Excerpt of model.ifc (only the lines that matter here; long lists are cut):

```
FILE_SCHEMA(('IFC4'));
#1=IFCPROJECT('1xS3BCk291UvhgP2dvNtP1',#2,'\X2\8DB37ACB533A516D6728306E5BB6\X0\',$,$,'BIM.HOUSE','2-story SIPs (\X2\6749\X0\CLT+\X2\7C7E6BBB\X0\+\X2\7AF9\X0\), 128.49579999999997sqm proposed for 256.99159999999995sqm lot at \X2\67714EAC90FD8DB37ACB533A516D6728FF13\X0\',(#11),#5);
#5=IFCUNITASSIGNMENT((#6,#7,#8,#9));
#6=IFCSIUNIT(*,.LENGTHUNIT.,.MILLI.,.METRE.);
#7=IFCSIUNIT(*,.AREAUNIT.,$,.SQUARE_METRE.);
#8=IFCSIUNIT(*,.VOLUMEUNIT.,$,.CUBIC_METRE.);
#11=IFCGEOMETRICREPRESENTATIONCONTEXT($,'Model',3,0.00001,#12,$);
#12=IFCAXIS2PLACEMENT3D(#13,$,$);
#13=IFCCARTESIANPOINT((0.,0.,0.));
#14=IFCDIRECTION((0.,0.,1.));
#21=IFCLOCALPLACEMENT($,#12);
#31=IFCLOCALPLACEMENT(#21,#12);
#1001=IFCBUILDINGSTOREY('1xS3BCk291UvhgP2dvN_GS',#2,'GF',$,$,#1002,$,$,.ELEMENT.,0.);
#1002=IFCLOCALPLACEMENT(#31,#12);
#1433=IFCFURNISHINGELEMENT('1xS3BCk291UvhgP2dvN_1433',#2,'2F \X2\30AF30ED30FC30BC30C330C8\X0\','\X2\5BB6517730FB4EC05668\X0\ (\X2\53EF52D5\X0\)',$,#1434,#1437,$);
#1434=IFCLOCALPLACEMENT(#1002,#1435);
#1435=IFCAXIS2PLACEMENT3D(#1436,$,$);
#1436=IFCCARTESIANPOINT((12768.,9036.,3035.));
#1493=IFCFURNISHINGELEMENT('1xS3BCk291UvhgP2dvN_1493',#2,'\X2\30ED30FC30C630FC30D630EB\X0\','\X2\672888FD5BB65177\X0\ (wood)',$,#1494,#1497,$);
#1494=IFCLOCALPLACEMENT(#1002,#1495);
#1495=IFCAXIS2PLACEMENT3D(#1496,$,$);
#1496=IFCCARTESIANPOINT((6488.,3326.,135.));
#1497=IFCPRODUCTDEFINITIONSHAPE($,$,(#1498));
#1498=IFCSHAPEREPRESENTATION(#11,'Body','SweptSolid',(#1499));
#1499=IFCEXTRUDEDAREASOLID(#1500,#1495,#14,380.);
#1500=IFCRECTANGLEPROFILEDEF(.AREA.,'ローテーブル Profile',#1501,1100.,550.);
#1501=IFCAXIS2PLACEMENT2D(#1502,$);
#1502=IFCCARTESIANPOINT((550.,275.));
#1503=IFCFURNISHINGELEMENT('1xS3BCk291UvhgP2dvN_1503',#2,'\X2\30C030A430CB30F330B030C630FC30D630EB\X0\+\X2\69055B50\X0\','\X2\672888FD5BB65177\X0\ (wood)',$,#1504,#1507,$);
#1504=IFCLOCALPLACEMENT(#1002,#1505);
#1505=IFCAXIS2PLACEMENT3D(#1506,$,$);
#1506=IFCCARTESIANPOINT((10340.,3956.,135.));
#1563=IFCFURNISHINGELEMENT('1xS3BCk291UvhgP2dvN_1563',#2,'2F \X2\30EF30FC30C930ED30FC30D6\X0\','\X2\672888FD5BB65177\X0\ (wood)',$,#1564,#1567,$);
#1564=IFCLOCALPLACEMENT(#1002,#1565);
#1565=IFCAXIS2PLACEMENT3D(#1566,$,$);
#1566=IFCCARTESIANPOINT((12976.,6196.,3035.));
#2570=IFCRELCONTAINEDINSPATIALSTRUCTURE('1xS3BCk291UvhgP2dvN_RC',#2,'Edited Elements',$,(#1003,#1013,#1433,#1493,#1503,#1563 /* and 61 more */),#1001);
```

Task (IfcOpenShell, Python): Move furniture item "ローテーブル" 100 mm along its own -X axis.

```python
import ifcopenshell
import ifcopenshell.api.geometry
import ifcopenshell.util.placement
import ifcopenshell.util.unit

model = ifcopenshell.open("model.ifc")
unit_scale = ifcopenshell.util.unit.calculate_unit_scale(model)

item = model.by_guid("1xS3BCk291UvhgP2dvN_1493")
matrix = ifcopenshell.util.placement.get_local_placement(item.ObjectPlacement)
matrix[:3, 3] -= matrix[:3, 0] * 0.1 / unit_scale
ifcopenshell.api.geometry.edit_object_placement(model, product=item, matrix=matrix, is_si=False)

print(ifcopenshell.util.placement.get_local_placement(item.ObjectPlacement).round(3) + 0.0)

model.write("model_v2.ifc")
```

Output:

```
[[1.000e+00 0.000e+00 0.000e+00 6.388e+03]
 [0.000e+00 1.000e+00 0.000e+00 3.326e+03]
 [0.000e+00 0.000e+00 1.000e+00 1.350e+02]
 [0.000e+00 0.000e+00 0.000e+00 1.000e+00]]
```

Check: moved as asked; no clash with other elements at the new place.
